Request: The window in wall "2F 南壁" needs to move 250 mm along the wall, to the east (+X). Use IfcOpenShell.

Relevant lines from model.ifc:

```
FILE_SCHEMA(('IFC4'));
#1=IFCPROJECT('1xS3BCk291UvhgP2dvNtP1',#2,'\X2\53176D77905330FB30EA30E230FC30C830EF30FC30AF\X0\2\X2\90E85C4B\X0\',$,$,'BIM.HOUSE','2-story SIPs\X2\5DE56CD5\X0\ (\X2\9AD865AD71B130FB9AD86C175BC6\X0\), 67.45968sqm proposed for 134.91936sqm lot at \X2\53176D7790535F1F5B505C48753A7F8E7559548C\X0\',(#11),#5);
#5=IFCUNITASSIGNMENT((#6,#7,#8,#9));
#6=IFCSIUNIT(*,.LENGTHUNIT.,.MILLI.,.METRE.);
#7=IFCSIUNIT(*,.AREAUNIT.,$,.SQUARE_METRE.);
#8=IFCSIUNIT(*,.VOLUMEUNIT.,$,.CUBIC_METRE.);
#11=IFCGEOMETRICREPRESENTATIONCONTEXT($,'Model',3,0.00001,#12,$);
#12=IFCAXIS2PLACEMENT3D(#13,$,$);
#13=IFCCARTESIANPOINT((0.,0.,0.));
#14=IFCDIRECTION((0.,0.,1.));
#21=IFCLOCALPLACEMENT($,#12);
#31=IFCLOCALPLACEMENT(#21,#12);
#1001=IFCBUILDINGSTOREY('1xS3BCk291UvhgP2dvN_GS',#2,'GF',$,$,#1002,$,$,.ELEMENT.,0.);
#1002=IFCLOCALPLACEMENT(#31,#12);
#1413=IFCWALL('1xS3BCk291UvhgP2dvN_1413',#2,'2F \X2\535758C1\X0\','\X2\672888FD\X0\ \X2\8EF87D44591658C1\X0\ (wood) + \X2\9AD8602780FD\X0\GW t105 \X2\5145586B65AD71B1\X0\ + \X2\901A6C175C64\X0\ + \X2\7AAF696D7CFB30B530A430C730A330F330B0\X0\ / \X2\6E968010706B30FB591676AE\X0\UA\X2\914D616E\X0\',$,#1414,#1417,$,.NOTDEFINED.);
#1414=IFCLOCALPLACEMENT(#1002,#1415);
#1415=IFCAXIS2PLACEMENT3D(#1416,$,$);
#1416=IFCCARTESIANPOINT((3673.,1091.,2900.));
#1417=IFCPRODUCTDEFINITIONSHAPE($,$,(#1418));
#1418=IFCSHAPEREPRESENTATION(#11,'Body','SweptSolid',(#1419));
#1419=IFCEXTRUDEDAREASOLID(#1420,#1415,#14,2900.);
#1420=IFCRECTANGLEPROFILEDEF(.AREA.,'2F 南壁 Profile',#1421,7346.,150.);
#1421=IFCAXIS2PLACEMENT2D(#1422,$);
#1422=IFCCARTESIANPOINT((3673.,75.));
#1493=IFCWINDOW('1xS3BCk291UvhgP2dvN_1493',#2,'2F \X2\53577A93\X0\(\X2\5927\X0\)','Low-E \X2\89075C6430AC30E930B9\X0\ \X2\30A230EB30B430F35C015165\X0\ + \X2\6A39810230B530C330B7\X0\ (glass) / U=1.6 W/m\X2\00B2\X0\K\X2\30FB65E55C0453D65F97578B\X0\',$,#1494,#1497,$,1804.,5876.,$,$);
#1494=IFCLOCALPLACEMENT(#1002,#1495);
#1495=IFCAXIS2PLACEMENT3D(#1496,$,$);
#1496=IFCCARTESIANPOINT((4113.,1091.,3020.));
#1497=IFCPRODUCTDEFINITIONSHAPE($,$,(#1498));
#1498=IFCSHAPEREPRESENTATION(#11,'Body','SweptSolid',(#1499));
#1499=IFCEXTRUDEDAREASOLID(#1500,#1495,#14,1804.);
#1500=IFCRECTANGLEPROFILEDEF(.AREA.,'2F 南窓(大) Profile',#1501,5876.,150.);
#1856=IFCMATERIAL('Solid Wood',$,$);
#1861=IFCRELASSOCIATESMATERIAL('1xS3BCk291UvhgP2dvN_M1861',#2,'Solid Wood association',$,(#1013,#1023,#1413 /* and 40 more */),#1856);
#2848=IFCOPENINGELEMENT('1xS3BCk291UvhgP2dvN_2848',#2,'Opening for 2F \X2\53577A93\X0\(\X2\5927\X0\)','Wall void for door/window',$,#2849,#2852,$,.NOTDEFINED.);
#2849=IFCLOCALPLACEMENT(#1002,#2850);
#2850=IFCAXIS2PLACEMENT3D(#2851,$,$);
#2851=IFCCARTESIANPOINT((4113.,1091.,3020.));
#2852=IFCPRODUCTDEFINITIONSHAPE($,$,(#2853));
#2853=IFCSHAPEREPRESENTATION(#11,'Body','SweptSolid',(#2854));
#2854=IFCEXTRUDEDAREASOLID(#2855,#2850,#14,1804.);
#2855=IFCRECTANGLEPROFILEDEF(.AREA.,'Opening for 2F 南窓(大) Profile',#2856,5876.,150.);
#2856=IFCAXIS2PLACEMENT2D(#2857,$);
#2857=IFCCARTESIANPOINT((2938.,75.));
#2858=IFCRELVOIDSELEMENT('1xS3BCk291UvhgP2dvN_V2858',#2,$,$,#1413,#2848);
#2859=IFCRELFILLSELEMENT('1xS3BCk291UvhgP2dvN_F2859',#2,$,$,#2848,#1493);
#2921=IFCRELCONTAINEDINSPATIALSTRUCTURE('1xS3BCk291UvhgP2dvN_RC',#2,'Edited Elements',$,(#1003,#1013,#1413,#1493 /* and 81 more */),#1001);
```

```python
import ifcopenshell
import ifcopenshell.api.geometry
import ifcopenshell.util.placement

model = ifcopenshell.open("model.ifc")

window = model.by_guid("1xS3BCk291UvhgP2dvN_1493")
opening = window.FillsVoids[0].RelatingOpeningElement
wall = opening.VoidsElements[0].RelatingBuildingElement

wall_matrix = ifcopenshell.util.placement.get_local_placement(wall.ObjectPlacement)
shift = wall_matrix[:3, 0] * 250.0
before = ifcopenshell.util.placement.get_local_placement(window.ObjectPlacement)[:3, 3].copy()

# The window is not placed relative to its opening, so move both.
for product in (opening, window):
    matrix = ifcopenshell.util.placement.get_local_placement(product.ObjectPlacement)
    matrix[:3, 3] += shift
    ifcopenshell.api.geometry.edit_object_placement(model, product=product, matrix=matrix, is_si=False)

after = ifcopenshell.util.placement.get_local_placement(window.ObjectPlacement)[:3, 3]
print("window moved by", (after - before).round(3) + 0.0)

model.write("model_edited.ifc")
```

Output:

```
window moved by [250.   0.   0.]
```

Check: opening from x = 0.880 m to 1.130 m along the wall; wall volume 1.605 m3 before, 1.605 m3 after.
